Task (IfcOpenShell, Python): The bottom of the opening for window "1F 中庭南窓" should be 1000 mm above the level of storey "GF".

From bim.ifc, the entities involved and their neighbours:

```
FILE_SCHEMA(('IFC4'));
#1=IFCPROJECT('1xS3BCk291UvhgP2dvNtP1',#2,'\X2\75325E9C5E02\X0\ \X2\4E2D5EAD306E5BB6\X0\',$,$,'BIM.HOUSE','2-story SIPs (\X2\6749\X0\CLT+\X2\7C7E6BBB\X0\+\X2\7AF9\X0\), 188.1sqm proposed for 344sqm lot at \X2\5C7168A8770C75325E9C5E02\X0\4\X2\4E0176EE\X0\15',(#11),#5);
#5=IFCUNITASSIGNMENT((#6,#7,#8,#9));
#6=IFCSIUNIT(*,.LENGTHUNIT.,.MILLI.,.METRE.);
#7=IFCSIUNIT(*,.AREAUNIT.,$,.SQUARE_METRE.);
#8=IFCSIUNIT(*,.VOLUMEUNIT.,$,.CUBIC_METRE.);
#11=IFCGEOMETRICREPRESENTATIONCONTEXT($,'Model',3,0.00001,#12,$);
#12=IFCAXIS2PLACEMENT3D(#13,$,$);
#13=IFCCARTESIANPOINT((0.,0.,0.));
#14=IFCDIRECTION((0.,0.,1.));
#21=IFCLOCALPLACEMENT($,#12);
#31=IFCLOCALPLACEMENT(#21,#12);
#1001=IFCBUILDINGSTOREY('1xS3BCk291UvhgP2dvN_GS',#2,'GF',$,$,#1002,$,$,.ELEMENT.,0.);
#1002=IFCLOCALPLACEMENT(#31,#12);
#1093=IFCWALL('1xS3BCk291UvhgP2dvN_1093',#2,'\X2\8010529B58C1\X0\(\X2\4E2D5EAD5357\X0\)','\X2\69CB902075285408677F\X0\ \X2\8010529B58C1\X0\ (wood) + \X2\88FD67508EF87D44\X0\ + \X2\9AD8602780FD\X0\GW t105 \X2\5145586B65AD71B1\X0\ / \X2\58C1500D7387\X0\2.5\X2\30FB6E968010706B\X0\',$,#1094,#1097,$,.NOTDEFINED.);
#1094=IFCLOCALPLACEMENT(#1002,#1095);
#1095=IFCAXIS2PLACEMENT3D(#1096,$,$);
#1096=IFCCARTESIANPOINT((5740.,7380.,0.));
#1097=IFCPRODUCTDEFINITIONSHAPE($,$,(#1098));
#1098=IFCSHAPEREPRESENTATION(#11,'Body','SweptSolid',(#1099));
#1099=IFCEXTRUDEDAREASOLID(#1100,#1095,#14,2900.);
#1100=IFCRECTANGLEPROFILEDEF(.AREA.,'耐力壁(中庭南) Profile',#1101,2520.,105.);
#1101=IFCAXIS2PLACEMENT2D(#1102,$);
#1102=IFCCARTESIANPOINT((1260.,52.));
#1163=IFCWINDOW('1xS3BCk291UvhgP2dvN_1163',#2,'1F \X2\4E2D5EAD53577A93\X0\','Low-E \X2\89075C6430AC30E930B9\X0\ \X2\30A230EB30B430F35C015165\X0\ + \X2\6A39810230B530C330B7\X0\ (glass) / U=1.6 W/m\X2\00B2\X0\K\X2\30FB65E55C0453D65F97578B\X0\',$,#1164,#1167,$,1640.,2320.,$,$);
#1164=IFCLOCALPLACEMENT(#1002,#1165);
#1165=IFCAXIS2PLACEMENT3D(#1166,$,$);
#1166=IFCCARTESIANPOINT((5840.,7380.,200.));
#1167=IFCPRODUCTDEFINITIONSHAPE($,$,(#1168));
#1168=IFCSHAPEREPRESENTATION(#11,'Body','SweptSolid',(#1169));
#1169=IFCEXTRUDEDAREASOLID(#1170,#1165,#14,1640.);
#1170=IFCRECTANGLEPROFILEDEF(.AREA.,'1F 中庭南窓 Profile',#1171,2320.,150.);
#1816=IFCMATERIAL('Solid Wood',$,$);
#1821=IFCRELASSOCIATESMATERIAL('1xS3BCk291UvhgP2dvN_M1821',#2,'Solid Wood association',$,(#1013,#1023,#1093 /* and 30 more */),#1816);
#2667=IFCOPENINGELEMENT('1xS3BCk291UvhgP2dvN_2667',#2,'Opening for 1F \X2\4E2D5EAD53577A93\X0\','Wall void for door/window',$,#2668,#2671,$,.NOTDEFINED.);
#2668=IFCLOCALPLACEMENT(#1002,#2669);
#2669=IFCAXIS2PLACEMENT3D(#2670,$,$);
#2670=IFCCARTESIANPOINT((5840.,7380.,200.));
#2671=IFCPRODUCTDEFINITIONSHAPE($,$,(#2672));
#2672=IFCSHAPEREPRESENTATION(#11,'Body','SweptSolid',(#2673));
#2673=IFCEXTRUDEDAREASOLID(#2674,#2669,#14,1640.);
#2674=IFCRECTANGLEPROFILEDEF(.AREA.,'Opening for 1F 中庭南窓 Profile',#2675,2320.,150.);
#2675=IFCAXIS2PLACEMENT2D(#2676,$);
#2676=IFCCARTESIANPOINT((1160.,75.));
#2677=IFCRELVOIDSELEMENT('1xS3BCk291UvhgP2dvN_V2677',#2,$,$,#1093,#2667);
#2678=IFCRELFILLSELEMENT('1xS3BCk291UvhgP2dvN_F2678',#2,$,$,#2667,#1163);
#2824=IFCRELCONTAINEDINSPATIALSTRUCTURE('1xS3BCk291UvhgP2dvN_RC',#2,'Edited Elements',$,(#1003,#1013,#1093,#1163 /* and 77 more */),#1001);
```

```python
import numpy as np
import ifcopenshell
import ifcopenshell.api.geometry
import ifcopenshell.geom
import ifcopenshell.util.element
import ifcopenshell.util.placement
import ifcopenshell.util.shape
import ifcopenshell.util.unit

model = ifcopenshell.open("bim.ifc")
unit_scale = ifcopenshell.util.unit.calculate_unit_scale(model)

window = model.by_guid("1xS3BCk291UvhgP2dvN_1163")
opening = window.FillsVoids[0].RelatingOpeningElement
storey = ifcopenshell.util.element.get_container(window, ifc_class="IfcBuildingStorey")
level = ifcopenshell.util.placement.get_local_placement(storey.ObjectPlacement)[2, 3]

# The opening's origin need not be at the sill, so measure its lowest point.
shape = ifcopenshell.geom.create_shape(ifcopenshell.geom.settings(), opening)
bottom = ifcopenshell.util.shape.get_shape_bottom_elevation(shape, shape.geometry) / unit_scale
dz = level + 1 / unit_scale - bottom

shift = np.array([0.0, 0.0, dz])
# The window is not placed relative to its opening, so move both.
for product in (opening, window):
    matrix = ifcopenshell.util.placement.get_local_placement(product.ObjectPlacement)
    matrix[:3, 3] += shift
    ifcopenshell.api.geometry.edit_object_placement(model, product=product, matrix=matrix, is_si=False)

print(f"moved by {dz * unit_scale:+.3f} m")

model.write("bim_updated.ifc")
```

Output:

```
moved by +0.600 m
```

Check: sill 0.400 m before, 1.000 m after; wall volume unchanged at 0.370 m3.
